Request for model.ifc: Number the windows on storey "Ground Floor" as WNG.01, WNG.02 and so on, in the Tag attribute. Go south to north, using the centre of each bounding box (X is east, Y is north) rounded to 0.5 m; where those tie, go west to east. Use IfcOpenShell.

First a look at what the model holds.

```python
import ifcopenshell
import ifcopenshell.util.element
import ifcopenshell.util.placement

model = ifcopenshell.open("model.ifc")
print(model.schema)
storey = next(s for s in model.by_type("IfcBuildingStorey") if s.Name == "Ground Floor")
windows = [e for e in ifcopenshell.util.element.get_decomposition(storey) if e.is_a("IfcWindow")]
for e in sorted(windows, key=lambda e: e.id()):
    origin = ifcopenshell.util.placement.get_local_placement(e.ObjectPlacement)[:3, 3]
    print(e.id(), e.Tag, e.Name, origin.round(2) + 0.0, sep=" | ")
```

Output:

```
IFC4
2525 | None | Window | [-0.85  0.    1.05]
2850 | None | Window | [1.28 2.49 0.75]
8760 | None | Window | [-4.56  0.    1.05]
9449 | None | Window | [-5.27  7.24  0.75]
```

```python
import ifcopenshell
import ifcopenshell.geom
import ifcopenshell.util.element
import ifcopenshell.util.shape

model = ifcopenshell.open("model.ifc")
settings = ifcopenshell.geom.settings()
settings.set("use-world-coords", True)


def centre(element):
    shape = ifcopenshell.geom.create_shape(settings, element)
    return ifcopenshell.util.shape.get_bbox_centroid(shape.geometry)


storey = next(s for s in model.by_type("IfcBuildingStorey") if s.Name == "Ground Floor")
windows = [e for e in ifcopenshell.util.element.get_decomposition(storey) if e.is_a("IfcWindow")]

# Insertion points can sit at a corner or the storey origin, so sort by the geometry (in metres).
centres = {e: centre(e) for e in windows}
windows.sort(key=lambda e: (round(centres[e][1] / 0.5), centres[e][0]))

for i, e in enumerate(windows, start=1):
    number = f"WNG.{i:02d}"
    e.Tag = number
    print(e.id(), number)

model.write("model_updated.ifc")
```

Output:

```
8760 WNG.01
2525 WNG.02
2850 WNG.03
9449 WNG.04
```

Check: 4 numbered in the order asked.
